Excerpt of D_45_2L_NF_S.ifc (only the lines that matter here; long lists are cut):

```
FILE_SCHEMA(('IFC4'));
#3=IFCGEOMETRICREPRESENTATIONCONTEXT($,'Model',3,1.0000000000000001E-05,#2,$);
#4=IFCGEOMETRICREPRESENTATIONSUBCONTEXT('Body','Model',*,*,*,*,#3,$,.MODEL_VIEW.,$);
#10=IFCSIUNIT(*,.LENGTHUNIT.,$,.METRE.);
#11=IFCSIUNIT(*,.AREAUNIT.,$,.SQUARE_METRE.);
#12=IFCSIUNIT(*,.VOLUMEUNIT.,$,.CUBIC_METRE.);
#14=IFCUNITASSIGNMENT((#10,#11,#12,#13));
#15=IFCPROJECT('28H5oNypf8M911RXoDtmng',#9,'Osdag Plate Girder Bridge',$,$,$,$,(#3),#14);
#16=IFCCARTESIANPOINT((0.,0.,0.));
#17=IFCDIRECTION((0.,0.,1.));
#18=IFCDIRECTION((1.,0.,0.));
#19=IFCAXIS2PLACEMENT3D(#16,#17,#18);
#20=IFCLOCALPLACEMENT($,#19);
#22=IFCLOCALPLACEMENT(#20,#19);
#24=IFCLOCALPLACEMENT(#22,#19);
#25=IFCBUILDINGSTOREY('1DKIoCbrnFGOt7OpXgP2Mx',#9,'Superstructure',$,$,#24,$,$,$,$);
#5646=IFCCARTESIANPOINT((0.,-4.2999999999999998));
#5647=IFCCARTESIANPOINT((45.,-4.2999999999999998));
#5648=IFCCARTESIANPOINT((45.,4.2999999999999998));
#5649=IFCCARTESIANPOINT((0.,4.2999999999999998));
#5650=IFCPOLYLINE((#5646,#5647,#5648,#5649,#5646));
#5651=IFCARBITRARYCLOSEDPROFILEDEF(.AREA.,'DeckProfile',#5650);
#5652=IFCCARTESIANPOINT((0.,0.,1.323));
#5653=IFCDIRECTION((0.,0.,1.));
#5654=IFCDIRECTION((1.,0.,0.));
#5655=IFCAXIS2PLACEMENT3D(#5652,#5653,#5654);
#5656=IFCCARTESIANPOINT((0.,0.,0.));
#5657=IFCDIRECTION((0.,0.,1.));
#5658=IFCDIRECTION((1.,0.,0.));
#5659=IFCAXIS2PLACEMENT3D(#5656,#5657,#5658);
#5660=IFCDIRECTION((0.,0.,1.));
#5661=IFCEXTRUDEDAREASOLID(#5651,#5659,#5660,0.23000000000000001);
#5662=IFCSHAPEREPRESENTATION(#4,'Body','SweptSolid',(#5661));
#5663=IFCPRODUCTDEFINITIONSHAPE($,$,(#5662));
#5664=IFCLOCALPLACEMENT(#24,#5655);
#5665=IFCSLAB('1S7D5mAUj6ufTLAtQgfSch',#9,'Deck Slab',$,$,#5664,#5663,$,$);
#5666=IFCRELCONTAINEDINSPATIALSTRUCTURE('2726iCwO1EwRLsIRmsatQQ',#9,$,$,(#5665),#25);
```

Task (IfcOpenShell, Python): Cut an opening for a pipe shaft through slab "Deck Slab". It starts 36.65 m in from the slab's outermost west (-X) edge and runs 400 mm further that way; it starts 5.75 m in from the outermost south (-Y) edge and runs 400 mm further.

```python
import numpy as np
import ifcopenshell
import ifcopenshell.api.feature
import ifcopenshell.api.geometry
import ifcopenshell.api.root
import ifcopenshell.geom
import ifcopenshell.util.placement
import ifcopenshell.util.representation
import ifcopenshell.util.shape
import ifcopenshell.util.unit

model = ifcopenshell.open("D_45_2L_NF_S.ifc")
unit_scale = ifcopenshell.util.unit.calculate_unit_scale(model)
settings = ifcopenshell.geom.settings()


def volume(element):
    """Net volume in cubic metres, openings subtracted."""
    shape = ifcopenshell.geom.create_shape(settings, element)
    return ifcopenshell.util.shape.get_volume(shape.geometry)


slab = model.by_id(5665)
before = volume(slab)

# Extent in the slab's own axes, in metres. The edges named are its -X and -Y sides.
slab_shape = ifcopenshell.geom.create_shape(settings, slab)
vertices = ifcopenshell.util.shape.get_vertices(slab_shape.geometry)
x_min, y_min, bottom = vertices.min(axis=0)
top = vertices[:, 2].max()

opening = ifcopenshell.api.root.create_entity(model, ifc_class="IfcOpeningElement", name="Pipe shaft opening", predefined_type="OPENING")
context = ifcopenshell.util.representation.get_context(model, "Model", "Body", "MODEL_VIEW")
width, depth = 0.4, 0.4
outline = [(0.0, 0.0), (width, 0.0), (width, depth), (0.0, depth), (0.0, 0.0)]
# Overshoot both faces by 50 mm so the cut is clean.
shape = ifcopenshell.api.geometry.add_slab_representation(
    model, context=context, depth=top - bottom + 0.1, polyline=outline
)
ifcopenshell.api.geometry.assign_representation(model, product=opening, representation=shape)

matrix = ifcopenshell.util.placement.get_local_placement(slab.ObjectPlacement)
matrix[:, 3] = matrix @ np.append(np.array([x_min + 36.65, y_min + 5.75, bottom - 0.05]) / unit_scale, 1.0)
ifcopenshell.api.geometry.edit_object_placement(model, product=opening, matrix=matrix, is_si=False)
ifcopenshell.api.feature.add_feature(model, feature=opening, element=slab)

after = volume(slab)

print(f"slab volume {before:.3f} -> {after:.3f} m3")

model.write("D_45_2L_NF_S_edited.ifc")
```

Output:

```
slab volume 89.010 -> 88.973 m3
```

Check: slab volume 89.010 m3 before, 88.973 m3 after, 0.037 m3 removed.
